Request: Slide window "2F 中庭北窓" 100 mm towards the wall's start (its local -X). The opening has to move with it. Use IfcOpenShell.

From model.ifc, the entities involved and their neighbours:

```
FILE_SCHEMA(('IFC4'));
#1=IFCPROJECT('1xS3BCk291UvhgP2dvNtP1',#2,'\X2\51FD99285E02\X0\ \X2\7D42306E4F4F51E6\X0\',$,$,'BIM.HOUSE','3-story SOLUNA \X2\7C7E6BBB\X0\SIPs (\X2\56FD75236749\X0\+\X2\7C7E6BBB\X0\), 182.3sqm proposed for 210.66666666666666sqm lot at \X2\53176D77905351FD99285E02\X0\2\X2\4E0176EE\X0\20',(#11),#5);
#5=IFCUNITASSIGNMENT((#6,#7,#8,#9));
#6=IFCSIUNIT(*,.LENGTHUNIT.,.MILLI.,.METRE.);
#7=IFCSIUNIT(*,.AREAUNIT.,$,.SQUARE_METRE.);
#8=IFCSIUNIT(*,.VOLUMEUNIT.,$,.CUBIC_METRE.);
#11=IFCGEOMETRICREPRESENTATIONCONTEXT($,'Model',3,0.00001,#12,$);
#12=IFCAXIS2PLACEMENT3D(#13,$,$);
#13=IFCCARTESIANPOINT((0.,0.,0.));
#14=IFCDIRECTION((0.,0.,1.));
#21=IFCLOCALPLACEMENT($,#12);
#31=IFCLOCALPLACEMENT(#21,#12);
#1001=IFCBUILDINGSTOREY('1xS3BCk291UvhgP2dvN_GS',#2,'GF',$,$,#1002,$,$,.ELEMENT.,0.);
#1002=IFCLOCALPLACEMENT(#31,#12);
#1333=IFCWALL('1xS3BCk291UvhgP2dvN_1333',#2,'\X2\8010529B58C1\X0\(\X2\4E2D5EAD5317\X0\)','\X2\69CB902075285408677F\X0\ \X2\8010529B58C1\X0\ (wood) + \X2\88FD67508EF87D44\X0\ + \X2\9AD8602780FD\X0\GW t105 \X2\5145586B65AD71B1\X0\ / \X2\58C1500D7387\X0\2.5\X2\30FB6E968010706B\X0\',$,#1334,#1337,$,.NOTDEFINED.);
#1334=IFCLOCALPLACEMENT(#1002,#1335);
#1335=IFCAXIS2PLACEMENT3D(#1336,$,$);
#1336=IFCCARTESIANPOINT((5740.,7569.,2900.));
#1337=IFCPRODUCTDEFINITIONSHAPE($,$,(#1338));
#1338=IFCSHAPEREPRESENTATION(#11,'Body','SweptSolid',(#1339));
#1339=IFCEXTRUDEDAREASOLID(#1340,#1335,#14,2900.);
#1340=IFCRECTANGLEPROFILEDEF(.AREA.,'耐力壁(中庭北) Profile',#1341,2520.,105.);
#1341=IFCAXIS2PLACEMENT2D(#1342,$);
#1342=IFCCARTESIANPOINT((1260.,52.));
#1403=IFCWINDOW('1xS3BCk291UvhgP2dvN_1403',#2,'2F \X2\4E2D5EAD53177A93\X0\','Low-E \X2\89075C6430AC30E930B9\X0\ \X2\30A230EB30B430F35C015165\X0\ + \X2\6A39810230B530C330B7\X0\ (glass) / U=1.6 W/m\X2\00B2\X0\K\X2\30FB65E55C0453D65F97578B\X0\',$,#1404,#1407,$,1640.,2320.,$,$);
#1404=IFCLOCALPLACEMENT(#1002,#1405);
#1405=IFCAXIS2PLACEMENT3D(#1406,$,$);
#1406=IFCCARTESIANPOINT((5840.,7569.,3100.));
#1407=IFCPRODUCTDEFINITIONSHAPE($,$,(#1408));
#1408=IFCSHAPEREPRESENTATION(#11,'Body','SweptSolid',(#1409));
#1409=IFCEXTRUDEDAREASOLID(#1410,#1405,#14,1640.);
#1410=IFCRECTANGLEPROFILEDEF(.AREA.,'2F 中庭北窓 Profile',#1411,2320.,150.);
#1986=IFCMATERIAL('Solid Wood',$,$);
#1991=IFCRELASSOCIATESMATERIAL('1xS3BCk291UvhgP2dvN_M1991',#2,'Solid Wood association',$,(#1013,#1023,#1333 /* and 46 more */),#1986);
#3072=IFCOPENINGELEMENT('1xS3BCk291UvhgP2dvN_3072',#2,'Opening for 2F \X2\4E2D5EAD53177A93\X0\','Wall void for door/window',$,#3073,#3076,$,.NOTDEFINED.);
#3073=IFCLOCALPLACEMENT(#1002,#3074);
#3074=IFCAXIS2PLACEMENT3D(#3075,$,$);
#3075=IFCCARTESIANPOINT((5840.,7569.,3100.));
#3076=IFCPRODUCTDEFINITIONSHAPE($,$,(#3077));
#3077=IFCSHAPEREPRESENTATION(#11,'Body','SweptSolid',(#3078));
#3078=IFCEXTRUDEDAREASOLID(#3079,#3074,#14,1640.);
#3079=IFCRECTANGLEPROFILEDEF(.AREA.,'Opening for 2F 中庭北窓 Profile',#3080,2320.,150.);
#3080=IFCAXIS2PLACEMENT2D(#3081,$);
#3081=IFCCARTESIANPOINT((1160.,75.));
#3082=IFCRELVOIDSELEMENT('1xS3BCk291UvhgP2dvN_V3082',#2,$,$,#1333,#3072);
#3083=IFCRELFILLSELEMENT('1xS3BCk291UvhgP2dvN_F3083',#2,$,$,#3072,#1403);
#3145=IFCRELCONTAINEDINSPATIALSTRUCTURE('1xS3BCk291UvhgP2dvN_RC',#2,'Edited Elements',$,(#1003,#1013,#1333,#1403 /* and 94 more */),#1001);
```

```python
import ifcopenshell
import ifcopenshell.api.geometry
import ifcopenshell.util.placement
import ifcopenshell.util.unit

model = ifcopenshell.open("model.ifc")
unit_scale = ifcopenshell.util.unit.calculate_unit_scale(model)

window = model.by_guid("1xS3BCk291UvhgP2dvN_1403")
opening = window.FillsVoids[0].RelatingOpeningElement
wall = opening.VoidsElements[0].RelatingBuildingElement

wall_matrix = ifcopenshell.util.placement.get_local_placement(wall.ObjectPlacement)
shift = wall_matrix[:3, 0] * -0.1 / unit_scale
before = ifcopenshell.util.placement.get_local_placement(window.ObjectPlacement)[:3, 3].copy()

# The window is not placed relative to its opening, so move both.
for product in (opening, window):
    matrix = ifcopenshell.util.placement.get_local_placement(product.ObjectPlacement)
    matrix[:3, 3] += shift
    ifcopenshell.api.geometry.edit_object_placement(model, product=product, matrix=matrix, is_si=False)

after = ifcopenshell.util.placement.get_local_placement(window.ObjectPlacement)[:3, 3]
print("window moved by", (after - before).round(3) + 0.0)

model.write("model_rev.ifc")
```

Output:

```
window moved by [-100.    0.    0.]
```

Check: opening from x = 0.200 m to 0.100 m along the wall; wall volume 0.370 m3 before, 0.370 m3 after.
